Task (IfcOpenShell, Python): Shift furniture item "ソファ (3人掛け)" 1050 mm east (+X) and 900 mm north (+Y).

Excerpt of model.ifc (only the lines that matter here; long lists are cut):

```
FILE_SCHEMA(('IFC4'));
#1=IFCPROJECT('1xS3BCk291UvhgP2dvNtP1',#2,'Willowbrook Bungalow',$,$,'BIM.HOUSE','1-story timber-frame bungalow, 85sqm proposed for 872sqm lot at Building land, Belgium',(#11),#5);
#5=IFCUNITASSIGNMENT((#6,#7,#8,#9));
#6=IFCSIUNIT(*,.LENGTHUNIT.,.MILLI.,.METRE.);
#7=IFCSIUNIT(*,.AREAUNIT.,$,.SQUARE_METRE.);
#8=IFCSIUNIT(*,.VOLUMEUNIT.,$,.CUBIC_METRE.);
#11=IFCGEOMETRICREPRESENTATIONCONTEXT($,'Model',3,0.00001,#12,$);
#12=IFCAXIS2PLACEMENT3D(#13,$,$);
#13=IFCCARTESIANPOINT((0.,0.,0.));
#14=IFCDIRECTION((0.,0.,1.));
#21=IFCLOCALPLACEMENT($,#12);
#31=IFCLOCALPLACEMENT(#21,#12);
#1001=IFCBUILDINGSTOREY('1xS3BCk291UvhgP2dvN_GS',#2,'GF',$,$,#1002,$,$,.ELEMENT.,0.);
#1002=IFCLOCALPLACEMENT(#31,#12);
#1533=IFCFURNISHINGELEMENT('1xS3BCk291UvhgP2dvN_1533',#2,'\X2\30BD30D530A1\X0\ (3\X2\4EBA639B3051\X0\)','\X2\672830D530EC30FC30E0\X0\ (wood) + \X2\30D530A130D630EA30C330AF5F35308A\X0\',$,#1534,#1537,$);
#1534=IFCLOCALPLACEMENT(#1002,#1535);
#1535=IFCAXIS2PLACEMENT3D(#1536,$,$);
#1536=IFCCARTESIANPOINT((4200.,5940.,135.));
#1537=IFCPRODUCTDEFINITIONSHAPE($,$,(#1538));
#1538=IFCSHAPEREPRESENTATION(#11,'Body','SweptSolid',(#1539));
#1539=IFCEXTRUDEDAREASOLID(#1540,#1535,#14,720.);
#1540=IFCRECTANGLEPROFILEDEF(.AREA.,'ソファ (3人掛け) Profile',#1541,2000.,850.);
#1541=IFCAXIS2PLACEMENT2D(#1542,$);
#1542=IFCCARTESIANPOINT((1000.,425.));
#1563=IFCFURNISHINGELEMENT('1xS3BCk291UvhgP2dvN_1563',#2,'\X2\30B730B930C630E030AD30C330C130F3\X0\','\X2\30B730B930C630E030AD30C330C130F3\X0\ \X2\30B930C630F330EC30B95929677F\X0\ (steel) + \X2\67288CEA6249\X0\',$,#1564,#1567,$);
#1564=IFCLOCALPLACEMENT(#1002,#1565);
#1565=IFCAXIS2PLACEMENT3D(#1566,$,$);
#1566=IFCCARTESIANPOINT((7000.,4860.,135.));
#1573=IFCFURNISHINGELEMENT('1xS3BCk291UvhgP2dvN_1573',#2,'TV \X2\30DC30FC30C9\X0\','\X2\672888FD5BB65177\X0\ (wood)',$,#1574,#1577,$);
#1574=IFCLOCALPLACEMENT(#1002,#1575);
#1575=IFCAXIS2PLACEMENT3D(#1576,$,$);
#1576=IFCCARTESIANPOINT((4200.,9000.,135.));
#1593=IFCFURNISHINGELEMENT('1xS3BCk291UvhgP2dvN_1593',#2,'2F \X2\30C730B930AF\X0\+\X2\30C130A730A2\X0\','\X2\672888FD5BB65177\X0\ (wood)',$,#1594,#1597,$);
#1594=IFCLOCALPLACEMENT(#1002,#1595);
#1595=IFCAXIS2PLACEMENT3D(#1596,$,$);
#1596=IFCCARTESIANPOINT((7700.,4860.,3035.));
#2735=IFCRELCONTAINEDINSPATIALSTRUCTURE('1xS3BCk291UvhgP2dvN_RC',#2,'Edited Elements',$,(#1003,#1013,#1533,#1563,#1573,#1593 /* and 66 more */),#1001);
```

```python
import ifcopenshell
import ifcopenshell.api.geometry
import ifcopenshell.util.placement

model = ifcopenshell.open("model.ifc")

item = model.by_guid("1xS3BCk291UvhgP2dvN_1533")
matrix = ifcopenshell.util.placement.get_local_placement(item.ObjectPlacement)
matrix[0, 3] += 1050.0
matrix[1, 3] += 900.0
ifcopenshell.api.geometry.edit_object_placement(model, product=item, matrix=matrix, is_si=False)

print(ifcopenshell.util.placement.get_local_placement(item.ObjectPlacement).round(3) + 0.0)

model.write("model_updated.ifc")
```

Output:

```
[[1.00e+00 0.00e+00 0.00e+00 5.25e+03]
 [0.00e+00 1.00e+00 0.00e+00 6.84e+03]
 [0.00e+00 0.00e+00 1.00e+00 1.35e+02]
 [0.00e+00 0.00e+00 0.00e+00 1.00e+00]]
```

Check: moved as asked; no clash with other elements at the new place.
